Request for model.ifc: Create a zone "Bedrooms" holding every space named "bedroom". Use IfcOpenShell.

First a look at what the model holds.

```python
import ifcopenshell

model = ifcopenshell.open("model.ifc")
print(model.schema)
seen = {}
for space in model.by_type("IfcSpace"):
    seen[space.LongName] = seen.get(space.LongName, 0) + 1
for name, count in sorted(seen.items(), key=str):
    print(count, "x", name)
print("zones:", [z.Name for z in model.by_type("IfcZone")][:20])
```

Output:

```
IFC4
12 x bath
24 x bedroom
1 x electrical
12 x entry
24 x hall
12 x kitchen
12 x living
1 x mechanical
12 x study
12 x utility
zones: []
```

```python
import ifcopenshell
import ifcopenshell.api.group
import ifcopenshell.api.root

model = ifcopenshell.open("model.ifc")

names = {"bedroom"}
spaces = [s for s in model.by_type("IfcSpace") if s.LongName in names]

zone = ifcopenshell.api.root.create_entity(model, ifc_class="IfcZone", name="Bedrooms")
ifcopenshell.api.group.assign_group(model, products=spaces, group=zone)
print(len(spaces), "spaces in", zone.Name)

model.write("model_updated.ifc")
```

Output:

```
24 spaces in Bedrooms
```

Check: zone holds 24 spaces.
